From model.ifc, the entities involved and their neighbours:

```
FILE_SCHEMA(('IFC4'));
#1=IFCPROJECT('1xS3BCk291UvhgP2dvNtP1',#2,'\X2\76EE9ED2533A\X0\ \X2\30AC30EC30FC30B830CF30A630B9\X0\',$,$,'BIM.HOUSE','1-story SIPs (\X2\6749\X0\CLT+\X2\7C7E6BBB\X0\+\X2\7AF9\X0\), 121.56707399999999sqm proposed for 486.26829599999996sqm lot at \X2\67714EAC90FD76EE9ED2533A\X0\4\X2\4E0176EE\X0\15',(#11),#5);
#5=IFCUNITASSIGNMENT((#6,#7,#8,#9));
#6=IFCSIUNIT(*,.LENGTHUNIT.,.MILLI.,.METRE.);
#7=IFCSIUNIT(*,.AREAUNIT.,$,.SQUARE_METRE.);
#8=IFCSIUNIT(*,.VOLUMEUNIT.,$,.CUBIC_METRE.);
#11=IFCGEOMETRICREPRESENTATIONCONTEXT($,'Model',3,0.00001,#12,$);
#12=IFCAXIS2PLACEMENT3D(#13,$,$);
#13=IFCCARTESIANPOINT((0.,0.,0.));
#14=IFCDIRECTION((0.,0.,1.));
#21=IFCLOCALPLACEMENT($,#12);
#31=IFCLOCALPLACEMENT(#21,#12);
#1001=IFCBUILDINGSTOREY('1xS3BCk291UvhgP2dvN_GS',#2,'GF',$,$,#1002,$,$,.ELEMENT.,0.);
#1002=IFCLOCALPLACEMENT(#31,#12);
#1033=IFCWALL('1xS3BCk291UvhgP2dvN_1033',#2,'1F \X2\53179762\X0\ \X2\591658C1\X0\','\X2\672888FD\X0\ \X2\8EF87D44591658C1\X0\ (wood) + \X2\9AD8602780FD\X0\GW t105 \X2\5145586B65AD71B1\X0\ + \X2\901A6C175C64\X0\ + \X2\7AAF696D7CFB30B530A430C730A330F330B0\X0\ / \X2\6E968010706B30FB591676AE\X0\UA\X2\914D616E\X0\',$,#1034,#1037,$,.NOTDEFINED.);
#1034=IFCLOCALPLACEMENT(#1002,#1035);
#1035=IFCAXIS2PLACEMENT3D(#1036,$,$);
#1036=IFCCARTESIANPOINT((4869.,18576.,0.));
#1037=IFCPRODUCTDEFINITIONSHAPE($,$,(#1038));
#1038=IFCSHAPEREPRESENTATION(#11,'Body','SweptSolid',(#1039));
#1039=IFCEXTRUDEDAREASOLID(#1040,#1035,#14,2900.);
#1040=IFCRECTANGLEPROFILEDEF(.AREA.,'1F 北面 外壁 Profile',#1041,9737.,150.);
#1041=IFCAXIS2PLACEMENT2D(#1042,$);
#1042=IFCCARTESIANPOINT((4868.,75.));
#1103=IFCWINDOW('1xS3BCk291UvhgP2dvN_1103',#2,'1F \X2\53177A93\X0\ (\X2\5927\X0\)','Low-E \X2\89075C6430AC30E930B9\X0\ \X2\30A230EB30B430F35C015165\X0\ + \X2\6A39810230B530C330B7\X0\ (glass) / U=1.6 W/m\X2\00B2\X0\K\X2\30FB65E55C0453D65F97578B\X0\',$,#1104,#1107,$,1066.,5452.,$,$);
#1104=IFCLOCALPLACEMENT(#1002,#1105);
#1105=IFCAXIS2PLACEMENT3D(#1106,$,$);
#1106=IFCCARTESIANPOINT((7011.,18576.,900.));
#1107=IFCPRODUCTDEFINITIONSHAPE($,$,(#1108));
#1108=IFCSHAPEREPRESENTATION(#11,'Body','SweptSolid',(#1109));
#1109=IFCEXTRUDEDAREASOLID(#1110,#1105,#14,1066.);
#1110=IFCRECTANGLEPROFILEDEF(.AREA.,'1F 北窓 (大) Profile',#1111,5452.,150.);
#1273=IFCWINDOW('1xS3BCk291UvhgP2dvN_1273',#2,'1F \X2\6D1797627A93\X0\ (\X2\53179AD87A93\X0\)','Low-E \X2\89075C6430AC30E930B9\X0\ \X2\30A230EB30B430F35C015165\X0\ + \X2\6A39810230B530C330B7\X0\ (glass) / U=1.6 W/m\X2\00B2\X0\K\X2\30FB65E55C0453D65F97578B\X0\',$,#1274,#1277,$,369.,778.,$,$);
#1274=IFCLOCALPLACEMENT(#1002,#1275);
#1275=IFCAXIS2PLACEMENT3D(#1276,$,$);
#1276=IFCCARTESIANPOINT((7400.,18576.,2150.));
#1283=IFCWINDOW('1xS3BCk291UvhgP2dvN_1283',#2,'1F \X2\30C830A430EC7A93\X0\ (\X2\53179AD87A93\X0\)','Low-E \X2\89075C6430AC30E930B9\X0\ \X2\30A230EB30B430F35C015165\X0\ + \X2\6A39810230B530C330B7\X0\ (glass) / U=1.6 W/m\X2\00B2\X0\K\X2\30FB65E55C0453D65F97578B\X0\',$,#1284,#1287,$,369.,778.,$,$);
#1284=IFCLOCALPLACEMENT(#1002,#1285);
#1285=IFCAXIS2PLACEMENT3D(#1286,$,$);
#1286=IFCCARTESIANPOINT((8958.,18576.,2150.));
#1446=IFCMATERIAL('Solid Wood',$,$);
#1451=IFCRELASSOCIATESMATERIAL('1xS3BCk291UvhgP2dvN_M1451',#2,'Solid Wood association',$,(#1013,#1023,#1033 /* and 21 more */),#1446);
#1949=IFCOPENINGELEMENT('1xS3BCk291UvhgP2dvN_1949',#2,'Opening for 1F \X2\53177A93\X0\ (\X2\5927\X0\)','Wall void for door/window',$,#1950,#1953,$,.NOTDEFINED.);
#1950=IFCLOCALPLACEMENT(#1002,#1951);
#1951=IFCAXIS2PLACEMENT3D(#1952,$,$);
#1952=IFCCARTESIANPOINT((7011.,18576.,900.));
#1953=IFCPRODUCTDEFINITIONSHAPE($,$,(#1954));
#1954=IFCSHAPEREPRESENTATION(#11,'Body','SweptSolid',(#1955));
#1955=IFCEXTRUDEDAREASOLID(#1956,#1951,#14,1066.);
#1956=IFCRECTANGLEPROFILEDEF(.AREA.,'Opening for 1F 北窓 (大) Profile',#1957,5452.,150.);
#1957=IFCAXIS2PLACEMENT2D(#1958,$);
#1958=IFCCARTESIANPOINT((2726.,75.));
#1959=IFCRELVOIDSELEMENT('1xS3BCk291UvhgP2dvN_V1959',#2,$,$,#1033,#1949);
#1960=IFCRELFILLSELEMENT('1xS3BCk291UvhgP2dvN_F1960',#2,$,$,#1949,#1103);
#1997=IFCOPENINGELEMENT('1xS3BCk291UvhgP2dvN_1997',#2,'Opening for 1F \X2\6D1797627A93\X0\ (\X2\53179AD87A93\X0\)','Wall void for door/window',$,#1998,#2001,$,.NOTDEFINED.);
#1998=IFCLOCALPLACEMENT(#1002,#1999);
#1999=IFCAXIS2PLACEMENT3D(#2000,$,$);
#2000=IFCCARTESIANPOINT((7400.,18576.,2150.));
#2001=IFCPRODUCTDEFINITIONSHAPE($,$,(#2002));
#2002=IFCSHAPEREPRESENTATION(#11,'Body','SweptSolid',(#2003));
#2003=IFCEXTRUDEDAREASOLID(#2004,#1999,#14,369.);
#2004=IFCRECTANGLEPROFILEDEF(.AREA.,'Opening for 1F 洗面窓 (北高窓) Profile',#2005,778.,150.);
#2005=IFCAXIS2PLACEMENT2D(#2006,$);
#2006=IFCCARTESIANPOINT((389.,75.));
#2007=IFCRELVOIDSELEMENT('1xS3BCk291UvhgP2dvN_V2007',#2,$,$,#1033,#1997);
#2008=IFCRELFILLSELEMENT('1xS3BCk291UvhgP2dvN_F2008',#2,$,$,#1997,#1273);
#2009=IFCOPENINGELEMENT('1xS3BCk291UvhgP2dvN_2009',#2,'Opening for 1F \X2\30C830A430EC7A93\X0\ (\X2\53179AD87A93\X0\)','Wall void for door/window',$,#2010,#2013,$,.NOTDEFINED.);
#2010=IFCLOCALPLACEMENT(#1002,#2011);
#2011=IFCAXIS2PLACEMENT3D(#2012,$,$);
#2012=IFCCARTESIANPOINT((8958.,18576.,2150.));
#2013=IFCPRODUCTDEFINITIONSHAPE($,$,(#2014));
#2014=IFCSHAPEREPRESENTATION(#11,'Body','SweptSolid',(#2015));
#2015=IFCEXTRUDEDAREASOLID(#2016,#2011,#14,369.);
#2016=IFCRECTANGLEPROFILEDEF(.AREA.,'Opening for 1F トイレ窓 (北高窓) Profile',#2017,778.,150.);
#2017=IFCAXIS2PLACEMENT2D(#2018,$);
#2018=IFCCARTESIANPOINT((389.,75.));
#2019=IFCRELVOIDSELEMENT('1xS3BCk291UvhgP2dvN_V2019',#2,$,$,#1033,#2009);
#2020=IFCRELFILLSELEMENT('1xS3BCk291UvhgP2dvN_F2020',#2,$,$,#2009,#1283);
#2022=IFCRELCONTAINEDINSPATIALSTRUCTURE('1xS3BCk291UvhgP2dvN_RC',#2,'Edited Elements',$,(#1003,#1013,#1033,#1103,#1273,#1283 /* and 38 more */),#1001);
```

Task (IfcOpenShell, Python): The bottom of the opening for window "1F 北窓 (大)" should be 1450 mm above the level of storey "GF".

```python
import numpy as np
import ifcopenshell
import ifcopenshell.api.geometry
import ifcopenshell.geom
import ifcopenshell.util.element
import ifcopenshell.util.placement
import ifcopenshell.util.shape
import ifcopenshell.util.unit

model = ifcopenshell.open("model.ifc")
unit_scale = ifcopenshell.util.unit.calculate_unit_scale(model)

window = model.by_guid("1xS3BCk291UvhgP2dvN_1103")
opening = window.FillsVoids[0].RelatingOpeningElement
storey = ifcopenshell.util.element.get_container(window, ifc_class="IfcBuildingStorey")
level = ifcopenshell.util.placement.get_local_placement(storey.ObjectPlacement)[2, 3]

# The opening's origin need not be at the sill, so measure its lowest point.
shape = ifcopenshell.geom.create_shape(ifcopenshell.geom.settings(), opening)
bottom = ifcopenshell.util.shape.get_shape_bottom_elevation(shape, shape.geometry) / unit_scale
dz = level + 1.45 / unit_scale - bottom

shift = np.array([0.0, 0.0, dz])
# The window is not placed relative to its opening, so move both.
for product in (opening, window):
    matrix = ifcopenshell.util.placement.get_local_placement(product.ObjectPlacement)
    matrix[:3, 3] += shift
    ifcopenshell.api.geometry.edit_object_placement(model, product=product, matrix=matrix, is_si=False)

print(f"moved by {dz * unit_scale:+.3f} m")

model.write("model_updated.ifc")
```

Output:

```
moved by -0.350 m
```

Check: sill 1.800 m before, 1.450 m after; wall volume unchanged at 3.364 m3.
